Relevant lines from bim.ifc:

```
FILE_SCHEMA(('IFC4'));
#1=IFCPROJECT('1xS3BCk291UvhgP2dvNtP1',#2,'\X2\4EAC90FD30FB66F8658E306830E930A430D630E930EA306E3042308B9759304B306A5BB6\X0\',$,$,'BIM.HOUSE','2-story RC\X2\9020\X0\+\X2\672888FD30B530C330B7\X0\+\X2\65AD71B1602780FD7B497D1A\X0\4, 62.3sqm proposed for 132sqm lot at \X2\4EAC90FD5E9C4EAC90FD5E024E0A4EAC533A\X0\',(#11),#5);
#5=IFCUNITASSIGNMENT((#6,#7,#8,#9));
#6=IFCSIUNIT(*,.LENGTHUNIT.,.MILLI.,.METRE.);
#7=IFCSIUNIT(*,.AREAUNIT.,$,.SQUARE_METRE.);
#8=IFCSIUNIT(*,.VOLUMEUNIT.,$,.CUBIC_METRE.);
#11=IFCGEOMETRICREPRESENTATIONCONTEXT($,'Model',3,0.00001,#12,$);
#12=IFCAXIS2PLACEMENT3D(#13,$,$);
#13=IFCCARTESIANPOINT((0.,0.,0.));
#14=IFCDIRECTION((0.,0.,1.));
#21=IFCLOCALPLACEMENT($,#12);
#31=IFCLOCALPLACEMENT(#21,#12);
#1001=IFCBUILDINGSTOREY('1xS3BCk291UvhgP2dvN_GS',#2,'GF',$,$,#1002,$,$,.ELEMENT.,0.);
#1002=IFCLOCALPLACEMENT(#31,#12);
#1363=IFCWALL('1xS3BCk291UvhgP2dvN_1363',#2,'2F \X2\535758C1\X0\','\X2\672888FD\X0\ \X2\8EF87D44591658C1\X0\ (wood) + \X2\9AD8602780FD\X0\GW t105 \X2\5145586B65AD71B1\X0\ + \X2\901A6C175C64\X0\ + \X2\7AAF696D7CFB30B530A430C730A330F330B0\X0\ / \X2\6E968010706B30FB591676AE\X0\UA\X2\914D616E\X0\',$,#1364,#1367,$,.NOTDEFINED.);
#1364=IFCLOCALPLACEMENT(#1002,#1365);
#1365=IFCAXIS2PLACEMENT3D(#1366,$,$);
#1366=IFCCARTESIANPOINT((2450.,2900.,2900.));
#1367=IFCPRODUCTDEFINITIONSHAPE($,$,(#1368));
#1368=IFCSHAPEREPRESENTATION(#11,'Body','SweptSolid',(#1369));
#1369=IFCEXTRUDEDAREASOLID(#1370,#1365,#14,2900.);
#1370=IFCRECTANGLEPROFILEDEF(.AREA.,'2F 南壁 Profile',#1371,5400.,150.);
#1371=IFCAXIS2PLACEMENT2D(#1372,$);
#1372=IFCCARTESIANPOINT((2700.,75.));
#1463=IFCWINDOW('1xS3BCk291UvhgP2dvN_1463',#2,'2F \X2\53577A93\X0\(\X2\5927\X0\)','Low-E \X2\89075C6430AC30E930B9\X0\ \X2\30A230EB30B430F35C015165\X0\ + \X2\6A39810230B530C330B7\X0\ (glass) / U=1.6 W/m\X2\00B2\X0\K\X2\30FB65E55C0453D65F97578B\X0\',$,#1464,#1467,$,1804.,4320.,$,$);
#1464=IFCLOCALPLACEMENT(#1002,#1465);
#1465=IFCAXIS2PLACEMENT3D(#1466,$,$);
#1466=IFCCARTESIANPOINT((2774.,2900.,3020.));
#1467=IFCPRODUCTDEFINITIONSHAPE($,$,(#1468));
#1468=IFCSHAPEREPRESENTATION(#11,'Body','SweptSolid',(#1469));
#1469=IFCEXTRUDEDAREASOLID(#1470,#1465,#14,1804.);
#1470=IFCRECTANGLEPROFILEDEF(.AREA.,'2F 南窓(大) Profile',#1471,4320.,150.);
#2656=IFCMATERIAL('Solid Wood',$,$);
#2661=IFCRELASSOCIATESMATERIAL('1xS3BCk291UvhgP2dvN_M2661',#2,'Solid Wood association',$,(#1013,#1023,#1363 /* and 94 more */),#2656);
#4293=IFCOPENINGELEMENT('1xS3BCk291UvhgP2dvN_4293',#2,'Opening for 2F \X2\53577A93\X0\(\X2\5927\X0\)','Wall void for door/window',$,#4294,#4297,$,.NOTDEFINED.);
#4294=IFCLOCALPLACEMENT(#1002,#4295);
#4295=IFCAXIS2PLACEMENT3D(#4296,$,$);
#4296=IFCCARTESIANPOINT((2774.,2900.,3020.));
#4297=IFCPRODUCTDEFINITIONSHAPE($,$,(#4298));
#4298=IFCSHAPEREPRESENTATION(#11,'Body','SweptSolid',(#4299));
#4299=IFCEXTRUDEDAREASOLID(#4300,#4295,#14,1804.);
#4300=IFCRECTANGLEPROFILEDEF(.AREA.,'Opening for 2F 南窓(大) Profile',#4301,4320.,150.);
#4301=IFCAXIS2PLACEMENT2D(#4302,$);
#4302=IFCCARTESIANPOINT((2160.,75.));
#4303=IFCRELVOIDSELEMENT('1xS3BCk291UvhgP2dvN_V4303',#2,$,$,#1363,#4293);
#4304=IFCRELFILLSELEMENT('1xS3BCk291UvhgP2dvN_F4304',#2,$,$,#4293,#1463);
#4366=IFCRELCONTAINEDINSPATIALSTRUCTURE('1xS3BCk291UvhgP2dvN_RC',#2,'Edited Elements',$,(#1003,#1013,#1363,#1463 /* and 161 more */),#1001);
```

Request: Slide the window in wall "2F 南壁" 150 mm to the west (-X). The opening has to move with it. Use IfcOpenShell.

```python
import ifcopenshell
import ifcopenshell.api.geometry
import ifcopenshell.util.placement
import ifcopenshell.util.unit

model = ifcopenshell.open("bim.ifc")
unit_scale = ifcopenshell.util.unit.calculate_unit_scale(model)

window = model.by_id(1463)
opening = window.FillsVoids[0].RelatingOpeningElement
wall = opening.VoidsElements[0].RelatingBuildingElement

wall_matrix = ifcopenshell.util.placement.get_local_placement(wall.ObjectPlacement)
shift = wall_matrix[:3, 0] * -0.15 / unit_scale
before = ifcopenshell.util.placement.get_local_placement(window.ObjectPlacement)[:3, 3].copy()

# The window is not placed relative to its opening, so move both.
for product in (opening, window):
    matrix = ifcopenshell.util.placement.get_local_placement(product.ObjectPlacement)
    matrix[:3, 3] += shift
    ifcopenshell.api.geometry.edit_object_placement(model, product=product, matrix=matrix, is_si=False)

after = ifcopenshell.util.placement.get_local_placement(window.ObjectPlacement)[:3, 3]
print("window moved by", (after - before).round(3) + 0.0)

model.write("bim_rev.ifc")
```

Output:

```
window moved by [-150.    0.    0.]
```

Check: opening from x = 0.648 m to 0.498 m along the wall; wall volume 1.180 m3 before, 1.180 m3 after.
